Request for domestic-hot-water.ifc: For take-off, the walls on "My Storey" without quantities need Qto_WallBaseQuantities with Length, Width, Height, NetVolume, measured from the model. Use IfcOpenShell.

First a look at what the model holds.

```python
import ifcopenshell
import ifcopenshell.util.element
import ifcopenshell.util.unit

model = ifcopenshell.open("domestic-hot-water.ifc")
print(model.schema)
for unit_type in ("LENGTHUNIT", "AREAUNIT", "VOLUMEUNIT"):
    print(unit_type, ifcopenshell.util.unit.calculate_unit_scale(model, unit_type))
storey = next(s for s in model.by_type("IfcBuildingStorey") if s.Name == "My Storey")
walls = [e for e in ifcopenshell.util.element.get_decomposition(storey) if e.is_a("IfcWall")]
for e in sorted(walls, key=lambda e: e.id()):
    print(e.id(), e.is_a(), e.Name, list(ifcopenshell.util.element.get_psets(e, qtos_only=True)), sep=" | ")
```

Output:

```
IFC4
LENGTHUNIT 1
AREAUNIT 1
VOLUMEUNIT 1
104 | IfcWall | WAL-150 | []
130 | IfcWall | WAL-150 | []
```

```python
import ifcopenshell
import ifcopenshell.api.pset
import ifcopenshell.geom
import ifcopenshell.util.element
import ifcopenshell.util.shape
import ifcopenshell.util.unit

model = ifcopenshell.open("domestic-hot-water.ifc")
unit_scale = ifcopenshell.util.unit.calculate_unit_scale(model)
volume_scale = ifcopenshell.util.unit.calculate_unit_scale(model, "VOLUMEUNIT")
settings = ifcopenshell.geom.settings()

storey = next(s for s in model.by_type("IfcBuildingStorey") if s.Name == "My Storey")
walls = [e for e in ifcopenshell.util.element.get_decomposition(storey) if e.is_a("IfcWall")]

for e in sorted(walls, key=lambda e: e.id()):
    if ifcopenshell.util.element.get_psets(e, qtos_only=True, should_inherit=False):
        continue
    # Geometry comes back in metres, in the element's own axes.
    shape = ifcopenshell.geom.create_shape(settings, e)
    values = {
        "Length": ifcopenshell.util.shape.get_x(shape.geometry) / unit_scale,
        "Width": ifcopenshell.util.shape.get_y(shape.geometry) / unit_scale,
        "Height": ifcopenshell.util.shape.get_z(shape.geometry) / unit_scale,
        "NetVolume": ifcopenshell.util.shape.get_volume(shape.geometry) / volume_scale,
    }
    qto = ifcopenshell.api.pset.add_qto(model, product=e, name="Qto_WallBaseQuantities")
    ifcopenshell.api.pset.edit_qto(model, qto=qto, properties=values)
    print(e.id(), {k: round(v, 3) for k, v in values.items()})

model.write("domestic-hot-water-out.ifc")
```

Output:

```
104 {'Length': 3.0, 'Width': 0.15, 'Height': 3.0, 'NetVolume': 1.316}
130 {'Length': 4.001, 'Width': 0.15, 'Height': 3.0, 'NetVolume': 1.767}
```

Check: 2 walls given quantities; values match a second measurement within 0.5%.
